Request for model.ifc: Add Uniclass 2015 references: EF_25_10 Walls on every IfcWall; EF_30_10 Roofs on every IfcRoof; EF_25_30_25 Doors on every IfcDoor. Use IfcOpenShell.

First a look at what the model holds.

```python
import ifcopenshell

model = ifcopenshell.open("model.ifc")
print(model.schema)
print("classifications:", [c.Name for c in model.by_type("IfcClassification")])
for ifc_class in ("IfcDoor", "IfcRoof", "IfcStair", "IfcWall", "IfcWindow"):
    print(ifc_class, len(model.by_type(ifc_class)))
```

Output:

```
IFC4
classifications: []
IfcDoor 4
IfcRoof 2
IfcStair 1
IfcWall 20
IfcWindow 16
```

```python
import ifcopenshell
import ifcopenshell.api.classification

model = ifcopenshell.open("model.ifc")

system = ifcopenshell.api.classification.add_classification(model, classification="Uniclass 2015")

codes = {
    "IfcWall": ("EF_25_10", "Walls"),
    "IfcRoof": ("EF_30_10", "Roofs"),
    "IfcDoor": ("EF_25_30_25", "Doors"),
}
for ifc_class, (code, name) in codes.items():
    products = model.by_type(ifc_class)
    ifcopenshell.api.classification.add_reference(
        model, products=products, classification=system, identification=code, name=name
    )
    print(code, len(products))

model.write("model_updated.ifc")
```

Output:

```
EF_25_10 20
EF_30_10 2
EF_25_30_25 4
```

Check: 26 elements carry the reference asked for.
